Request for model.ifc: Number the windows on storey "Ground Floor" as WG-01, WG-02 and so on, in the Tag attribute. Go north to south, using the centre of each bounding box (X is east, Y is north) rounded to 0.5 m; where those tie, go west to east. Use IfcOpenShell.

First a look at what the model holds.

```python
import ifcopenshell
import ifcopenshell.util.element
import ifcopenshell.util.placement

model = ifcopenshell.open("model.ifc")
print(model.schema)
storey = next(s for s in model.by_type("IfcBuildingStorey") if s.Name == "Ground Floor")
windows = [e for e in ifcopenshell.util.element.get_decomposition(storey) if e.is_a("IfcWindow")]
for e in sorted(windows, key=lambda e: e.id()):
    origin = ifcopenshell.util.placement.get_local_placement(e.ObjectPlacement)[:3, 3]
    print(e.id(), e.Tag, e.Name, origin.round(2) + 0.0, sep=" | ")
```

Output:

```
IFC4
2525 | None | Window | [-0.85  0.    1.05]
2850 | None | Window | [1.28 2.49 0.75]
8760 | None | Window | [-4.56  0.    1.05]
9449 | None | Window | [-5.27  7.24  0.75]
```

```python
import ifcopenshell
import ifcopenshell.geom
import ifcopenshell.util.element
import ifcopenshell.util.shape

model = ifcopenshell.open("model.ifc")
settings = ifcopenshell.geom.settings()
settings.set("use-world-coords", True)


def centre(element):
    shape = ifcopenshell.geom.create_shape(settings, element)
    return ifcopenshell.util.shape.get_bbox_centroid(shape.geometry)


storey = next(s for s in model.by_type("IfcBuildingStorey") if s.Name == "Ground Floor")
windows = [e for e in ifcopenshell.util.element.get_decomposition(storey) if e.is_a("IfcWindow")]

# Insertion points can sit at a corner or the storey origin, so sort by the geometry (in metres).
centres = {e: centre(e) for e in windows}
windows.sort(key=lambda e: (-round(centres[e][1] / 0.5), centres[e][0]))

for i, e in enumerate(windows, start=1):
    number = f"WG-{i:02d}"
    e.Tag = number
    print(e.id(), number)

model.write("model_edited.ifc")
```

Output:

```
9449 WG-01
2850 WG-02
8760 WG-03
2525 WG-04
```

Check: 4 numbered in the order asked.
